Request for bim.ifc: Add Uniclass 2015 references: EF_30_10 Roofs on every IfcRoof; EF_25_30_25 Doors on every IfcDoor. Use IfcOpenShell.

First a look at what the model holds.

```python
import ifcopenshell

model = ifcopenshell.open("bim.ifc")
print(model.schema)
print("classifications:", [c.Name for c in model.by_type("IfcClassification")])
for ifc_class in ("IfcDoor", "IfcRoof", "IfcStair", "IfcWall", "IfcWindow"):
    print(ifc_class, len(model.by_type(ifc_class)))
```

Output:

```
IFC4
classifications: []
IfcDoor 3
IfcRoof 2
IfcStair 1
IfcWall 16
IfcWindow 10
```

```python
import ifcopenshell
import ifcopenshell.api.classification

model = ifcopenshell.open("bim.ifc")

system = ifcopenshell.api.classification.add_classification(model, classification="Uniclass 2015")

codes = {
    "IfcRoof": ("EF_30_10", "Roofs"),
    "IfcDoor": ("EF_25_30_25", "Doors"),
}
for ifc_class, (code, name) in codes.items():
    products = model.by_type(ifc_class)
    ifcopenshell.api.classification.add_reference(
        model, products=products, classification=system, identification=code, name=name
    )
    print(code, len(products))

model.write("bim_updated.ifc")
```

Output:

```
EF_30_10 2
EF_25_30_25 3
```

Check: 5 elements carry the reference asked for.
